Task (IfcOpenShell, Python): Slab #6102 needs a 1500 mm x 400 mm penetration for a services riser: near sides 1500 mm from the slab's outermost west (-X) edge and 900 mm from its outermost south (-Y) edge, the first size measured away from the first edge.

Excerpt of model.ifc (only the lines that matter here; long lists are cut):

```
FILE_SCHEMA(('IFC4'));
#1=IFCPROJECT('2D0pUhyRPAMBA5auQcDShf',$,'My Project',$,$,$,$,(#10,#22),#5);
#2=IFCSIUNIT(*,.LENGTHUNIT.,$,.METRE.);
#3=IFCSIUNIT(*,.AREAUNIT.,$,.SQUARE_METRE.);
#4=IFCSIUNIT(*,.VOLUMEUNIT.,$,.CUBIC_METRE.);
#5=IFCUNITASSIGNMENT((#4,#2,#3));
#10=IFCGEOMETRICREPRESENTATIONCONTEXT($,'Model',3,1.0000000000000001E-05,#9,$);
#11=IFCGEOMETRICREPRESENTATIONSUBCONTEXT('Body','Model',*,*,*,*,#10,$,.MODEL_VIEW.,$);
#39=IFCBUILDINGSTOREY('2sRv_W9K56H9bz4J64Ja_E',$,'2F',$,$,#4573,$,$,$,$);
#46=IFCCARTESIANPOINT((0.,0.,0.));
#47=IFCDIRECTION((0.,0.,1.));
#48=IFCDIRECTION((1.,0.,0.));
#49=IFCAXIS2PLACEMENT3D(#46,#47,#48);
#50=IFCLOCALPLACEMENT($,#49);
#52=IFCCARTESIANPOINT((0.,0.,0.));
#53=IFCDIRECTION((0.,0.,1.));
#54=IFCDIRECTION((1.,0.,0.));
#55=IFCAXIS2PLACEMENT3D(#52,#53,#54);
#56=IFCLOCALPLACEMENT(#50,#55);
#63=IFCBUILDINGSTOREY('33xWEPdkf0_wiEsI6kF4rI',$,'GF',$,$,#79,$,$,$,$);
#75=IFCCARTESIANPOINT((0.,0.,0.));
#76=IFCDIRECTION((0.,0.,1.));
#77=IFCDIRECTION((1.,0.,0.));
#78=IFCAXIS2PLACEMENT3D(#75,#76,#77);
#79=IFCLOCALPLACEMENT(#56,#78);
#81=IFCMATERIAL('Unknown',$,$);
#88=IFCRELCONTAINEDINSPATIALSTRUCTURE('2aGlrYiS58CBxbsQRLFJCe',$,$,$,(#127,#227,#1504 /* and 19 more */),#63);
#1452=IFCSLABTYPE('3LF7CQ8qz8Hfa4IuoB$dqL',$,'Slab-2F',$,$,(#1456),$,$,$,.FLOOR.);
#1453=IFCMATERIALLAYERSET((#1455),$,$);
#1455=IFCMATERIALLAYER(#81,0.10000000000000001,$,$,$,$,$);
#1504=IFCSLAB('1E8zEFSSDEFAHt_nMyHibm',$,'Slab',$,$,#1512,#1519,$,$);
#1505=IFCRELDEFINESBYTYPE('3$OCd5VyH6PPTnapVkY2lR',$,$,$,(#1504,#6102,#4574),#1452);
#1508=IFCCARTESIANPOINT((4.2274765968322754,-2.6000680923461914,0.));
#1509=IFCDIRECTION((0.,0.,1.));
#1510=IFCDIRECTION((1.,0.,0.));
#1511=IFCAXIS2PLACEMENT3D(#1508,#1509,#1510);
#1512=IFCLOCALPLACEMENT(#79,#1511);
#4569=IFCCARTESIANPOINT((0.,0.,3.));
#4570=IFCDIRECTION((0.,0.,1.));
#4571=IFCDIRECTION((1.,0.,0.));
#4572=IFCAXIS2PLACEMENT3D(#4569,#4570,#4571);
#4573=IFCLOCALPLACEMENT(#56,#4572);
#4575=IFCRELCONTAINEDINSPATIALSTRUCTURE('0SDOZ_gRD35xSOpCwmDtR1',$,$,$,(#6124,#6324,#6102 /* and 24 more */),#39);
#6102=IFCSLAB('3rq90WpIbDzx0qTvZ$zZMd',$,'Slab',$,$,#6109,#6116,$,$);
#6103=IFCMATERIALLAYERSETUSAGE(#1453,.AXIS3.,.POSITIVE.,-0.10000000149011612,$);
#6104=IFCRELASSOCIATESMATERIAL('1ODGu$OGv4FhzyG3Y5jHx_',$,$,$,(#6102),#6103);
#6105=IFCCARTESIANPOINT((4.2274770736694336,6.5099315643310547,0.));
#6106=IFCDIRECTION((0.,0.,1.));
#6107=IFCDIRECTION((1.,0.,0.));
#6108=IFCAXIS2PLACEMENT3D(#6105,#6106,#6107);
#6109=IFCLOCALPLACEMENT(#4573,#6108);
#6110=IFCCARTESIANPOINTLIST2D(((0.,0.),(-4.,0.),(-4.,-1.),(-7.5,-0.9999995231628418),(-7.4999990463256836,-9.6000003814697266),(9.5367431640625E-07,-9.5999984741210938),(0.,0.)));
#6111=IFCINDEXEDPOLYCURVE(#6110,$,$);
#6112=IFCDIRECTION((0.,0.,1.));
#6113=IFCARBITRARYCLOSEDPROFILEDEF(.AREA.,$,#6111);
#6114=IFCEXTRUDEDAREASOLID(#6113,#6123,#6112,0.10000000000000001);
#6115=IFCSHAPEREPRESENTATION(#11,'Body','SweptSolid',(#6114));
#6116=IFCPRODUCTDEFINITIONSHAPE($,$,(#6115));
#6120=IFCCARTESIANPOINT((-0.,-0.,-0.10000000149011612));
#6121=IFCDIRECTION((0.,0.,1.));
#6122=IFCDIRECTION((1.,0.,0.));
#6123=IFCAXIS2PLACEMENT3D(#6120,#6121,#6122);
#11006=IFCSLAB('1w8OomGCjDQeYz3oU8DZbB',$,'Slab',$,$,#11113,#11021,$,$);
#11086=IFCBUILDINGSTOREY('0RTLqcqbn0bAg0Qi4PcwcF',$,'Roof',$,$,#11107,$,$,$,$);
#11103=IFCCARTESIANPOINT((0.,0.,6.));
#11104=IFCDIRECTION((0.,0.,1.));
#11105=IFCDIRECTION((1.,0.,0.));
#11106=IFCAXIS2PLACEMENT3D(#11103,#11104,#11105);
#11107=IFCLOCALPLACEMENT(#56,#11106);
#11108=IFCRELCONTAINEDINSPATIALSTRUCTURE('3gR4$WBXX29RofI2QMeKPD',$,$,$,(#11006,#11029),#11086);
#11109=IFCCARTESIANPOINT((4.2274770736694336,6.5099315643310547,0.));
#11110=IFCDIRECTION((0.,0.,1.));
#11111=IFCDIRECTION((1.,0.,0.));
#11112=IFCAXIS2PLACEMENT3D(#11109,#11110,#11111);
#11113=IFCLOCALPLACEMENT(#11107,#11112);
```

```python
import numpy as np
import ifcopenshell
import ifcopenshell.api.feature
import ifcopenshell.api.geometry
import ifcopenshell.api.root
import ifcopenshell.geom
import ifcopenshell.util.placement
import ifcopenshell.util.representation
import ifcopenshell.util.shape
import ifcopenshell.util.unit

model = ifcopenshell.open("model.ifc")
unit_scale = ifcopenshell.util.unit.calculate_unit_scale(model)
settings = ifcopenshell.geom.settings()


def volume(element):
    """Net volume in cubic metres, openings subtracted."""
    shape = ifcopenshell.geom.create_shape(settings, element)
    return ifcopenshell.util.shape.get_volume(shape.geometry)


slab = model.by_id(6102)
before = volume(slab)

# Extent in the slab's own axes, in metres. The edges named are its -X and -Y sides.
slab_shape = ifcopenshell.geom.create_shape(settings, slab)
vertices = ifcopenshell.util.shape.get_vertices(slab_shape.geometry)
x_min, y_min, bottom = vertices.min(axis=0)
top = vertices[:, 2].max()

opening = ifcopenshell.api.root.create_entity(model, ifc_class="IfcOpeningElement", name="Services riser opening", predefined_type="OPENING")
context = ifcopenshell.util.representation.get_context(model, "Model", "Body", "MODEL_VIEW")
width, depth = 1.5, 0.4
outline = [(0.0, 0.0), (width, 0.0), (width, depth), (0.0, depth), (0.0, 0.0)]
# Overshoot both faces by 50 mm so the cut is clean.
shape = ifcopenshell.api.geometry.add_slab_representation(
    model, context=context, depth=top - bottom + 0.1, polyline=outline
)
ifcopenshell.api.geometry.assign_representation(model, product=opening, representation=shape)

matrix = ifcopenshell.util.placement.get_local_placement(slab.ObjectPlacement)
matrix[:, 3] = matrix @ np.append(np.array([x_min + 1.5, y_min + 0.9, bottom - 0.05]) / unit_scale, 1.0)
ifcopenshell.api.geometry.edit_object_placement(model, product=opening, matrix=matrix, is_si=False)
ifcopenshell.api.feature.add_feature(model, feature=opening, element=slab)

after = volume(slab)

print(f"slab volume {before:.3f} -> {after:.3f} m3")

model.write("model_updated.ifc")
```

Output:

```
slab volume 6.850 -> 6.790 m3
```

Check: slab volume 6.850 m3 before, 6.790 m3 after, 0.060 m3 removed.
